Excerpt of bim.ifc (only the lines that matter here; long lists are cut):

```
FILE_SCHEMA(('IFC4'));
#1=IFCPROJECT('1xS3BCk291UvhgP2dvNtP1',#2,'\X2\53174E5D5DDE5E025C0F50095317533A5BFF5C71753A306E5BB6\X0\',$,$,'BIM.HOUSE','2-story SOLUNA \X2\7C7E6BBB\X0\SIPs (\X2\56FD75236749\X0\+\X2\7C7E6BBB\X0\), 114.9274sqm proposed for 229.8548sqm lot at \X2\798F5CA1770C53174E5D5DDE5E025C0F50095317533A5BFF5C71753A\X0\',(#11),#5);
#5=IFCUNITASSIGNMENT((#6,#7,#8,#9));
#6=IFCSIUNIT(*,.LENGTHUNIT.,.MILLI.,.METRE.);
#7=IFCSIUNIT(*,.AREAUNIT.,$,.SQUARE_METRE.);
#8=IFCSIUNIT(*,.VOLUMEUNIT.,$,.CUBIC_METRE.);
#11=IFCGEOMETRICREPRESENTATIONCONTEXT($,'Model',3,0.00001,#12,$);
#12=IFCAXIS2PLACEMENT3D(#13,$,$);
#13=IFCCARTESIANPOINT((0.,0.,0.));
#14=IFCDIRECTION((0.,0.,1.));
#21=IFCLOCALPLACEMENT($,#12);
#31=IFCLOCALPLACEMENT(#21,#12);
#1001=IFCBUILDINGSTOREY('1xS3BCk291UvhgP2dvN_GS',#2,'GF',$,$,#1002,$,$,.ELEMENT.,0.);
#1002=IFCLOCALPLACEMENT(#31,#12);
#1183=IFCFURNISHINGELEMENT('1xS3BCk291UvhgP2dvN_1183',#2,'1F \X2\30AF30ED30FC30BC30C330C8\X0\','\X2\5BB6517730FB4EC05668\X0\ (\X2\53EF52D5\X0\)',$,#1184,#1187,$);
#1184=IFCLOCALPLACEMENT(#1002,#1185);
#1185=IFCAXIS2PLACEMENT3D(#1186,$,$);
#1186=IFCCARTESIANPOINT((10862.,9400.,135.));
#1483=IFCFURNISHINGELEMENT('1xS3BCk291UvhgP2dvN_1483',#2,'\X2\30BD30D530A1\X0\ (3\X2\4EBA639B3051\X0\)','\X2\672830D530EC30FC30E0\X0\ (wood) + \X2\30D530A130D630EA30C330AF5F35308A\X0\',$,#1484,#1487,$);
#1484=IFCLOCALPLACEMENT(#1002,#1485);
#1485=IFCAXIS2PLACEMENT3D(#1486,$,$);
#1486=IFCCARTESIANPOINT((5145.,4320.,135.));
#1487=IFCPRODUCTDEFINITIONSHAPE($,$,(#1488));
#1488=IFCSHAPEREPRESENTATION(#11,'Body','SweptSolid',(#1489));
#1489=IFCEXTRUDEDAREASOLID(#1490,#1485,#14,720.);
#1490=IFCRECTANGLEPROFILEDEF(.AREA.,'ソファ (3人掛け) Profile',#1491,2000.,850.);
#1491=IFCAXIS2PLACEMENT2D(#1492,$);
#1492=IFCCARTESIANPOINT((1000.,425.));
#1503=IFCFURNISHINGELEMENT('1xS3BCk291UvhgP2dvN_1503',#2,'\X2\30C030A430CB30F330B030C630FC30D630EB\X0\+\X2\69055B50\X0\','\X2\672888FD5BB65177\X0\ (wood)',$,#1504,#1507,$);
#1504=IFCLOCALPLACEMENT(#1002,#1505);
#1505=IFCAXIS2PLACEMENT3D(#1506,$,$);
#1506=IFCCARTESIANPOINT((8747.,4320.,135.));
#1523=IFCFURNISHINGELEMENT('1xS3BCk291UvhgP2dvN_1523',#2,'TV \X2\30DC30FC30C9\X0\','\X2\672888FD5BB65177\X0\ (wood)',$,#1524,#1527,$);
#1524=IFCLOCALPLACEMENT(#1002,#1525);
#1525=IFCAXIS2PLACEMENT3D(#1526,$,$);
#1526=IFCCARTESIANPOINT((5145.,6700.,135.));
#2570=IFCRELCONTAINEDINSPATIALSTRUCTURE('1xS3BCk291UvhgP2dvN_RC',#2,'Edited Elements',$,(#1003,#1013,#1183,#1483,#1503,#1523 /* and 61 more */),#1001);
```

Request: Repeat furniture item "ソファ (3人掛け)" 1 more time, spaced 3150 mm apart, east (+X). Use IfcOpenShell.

```python
import numpy as np
import ifcopenshell
import ifcopenshell.api.geometry
import ifcopenshell.api.root
import ifcopenshell.util.element
import ifcopenshell.util.placement
import ifcopenshell.util.unit

model = ifcopenshell.open("bim.ifc")
unit_scale = ifcopenshell.util.unit.calculate_unit_scale(model)


def reuse_history(source, copy):
    """copy_class also copies each property set's owner history, people and application; keep the originals."""
    for rel in copy.IsDefinedBy:
        if rel.is_a("IfcRelDefinesByProperties") and (history := rel.RelatingPropertyDefinition.OwnerHistory):
            rel.RelatingPropertyDefinition.OwnerHistory = source.OwnerHistory
            ifcopenshell.util.element.remove_deep2(model, history)


source = model.by_guid("1xS3BCk291UvhgP2dvN_1483")
base = ifcopenshell.util.placement.get_local_placement(source.ObjectPlacement)
step = np.array([1.0, 0.0, 0.0]) * 3.15 / unit_scale

for i in range(1, 2):
    copy = ifcopenshell.api.root.copy_class(model, product=source)
    copy.Representation = ifcopenshell.util.element.copy_deep(
        model, source.Representation, exclude=["IfcGeometricRepresentationContext", "IfcRepresentationMap"]
    )
    reuse_history(source, copy)
    matrix = base.copy()
    matrix[:3, 3] += i * step
    print("added at", matrix[:3, 3].round(3) + 0.0)
    ifcopenshell.api.geometry.edit_object_placement(model, product=copy, matrix=matrix, is_si=False)

model.write("bim_updated.ifc")
```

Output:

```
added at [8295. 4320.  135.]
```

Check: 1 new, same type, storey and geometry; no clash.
